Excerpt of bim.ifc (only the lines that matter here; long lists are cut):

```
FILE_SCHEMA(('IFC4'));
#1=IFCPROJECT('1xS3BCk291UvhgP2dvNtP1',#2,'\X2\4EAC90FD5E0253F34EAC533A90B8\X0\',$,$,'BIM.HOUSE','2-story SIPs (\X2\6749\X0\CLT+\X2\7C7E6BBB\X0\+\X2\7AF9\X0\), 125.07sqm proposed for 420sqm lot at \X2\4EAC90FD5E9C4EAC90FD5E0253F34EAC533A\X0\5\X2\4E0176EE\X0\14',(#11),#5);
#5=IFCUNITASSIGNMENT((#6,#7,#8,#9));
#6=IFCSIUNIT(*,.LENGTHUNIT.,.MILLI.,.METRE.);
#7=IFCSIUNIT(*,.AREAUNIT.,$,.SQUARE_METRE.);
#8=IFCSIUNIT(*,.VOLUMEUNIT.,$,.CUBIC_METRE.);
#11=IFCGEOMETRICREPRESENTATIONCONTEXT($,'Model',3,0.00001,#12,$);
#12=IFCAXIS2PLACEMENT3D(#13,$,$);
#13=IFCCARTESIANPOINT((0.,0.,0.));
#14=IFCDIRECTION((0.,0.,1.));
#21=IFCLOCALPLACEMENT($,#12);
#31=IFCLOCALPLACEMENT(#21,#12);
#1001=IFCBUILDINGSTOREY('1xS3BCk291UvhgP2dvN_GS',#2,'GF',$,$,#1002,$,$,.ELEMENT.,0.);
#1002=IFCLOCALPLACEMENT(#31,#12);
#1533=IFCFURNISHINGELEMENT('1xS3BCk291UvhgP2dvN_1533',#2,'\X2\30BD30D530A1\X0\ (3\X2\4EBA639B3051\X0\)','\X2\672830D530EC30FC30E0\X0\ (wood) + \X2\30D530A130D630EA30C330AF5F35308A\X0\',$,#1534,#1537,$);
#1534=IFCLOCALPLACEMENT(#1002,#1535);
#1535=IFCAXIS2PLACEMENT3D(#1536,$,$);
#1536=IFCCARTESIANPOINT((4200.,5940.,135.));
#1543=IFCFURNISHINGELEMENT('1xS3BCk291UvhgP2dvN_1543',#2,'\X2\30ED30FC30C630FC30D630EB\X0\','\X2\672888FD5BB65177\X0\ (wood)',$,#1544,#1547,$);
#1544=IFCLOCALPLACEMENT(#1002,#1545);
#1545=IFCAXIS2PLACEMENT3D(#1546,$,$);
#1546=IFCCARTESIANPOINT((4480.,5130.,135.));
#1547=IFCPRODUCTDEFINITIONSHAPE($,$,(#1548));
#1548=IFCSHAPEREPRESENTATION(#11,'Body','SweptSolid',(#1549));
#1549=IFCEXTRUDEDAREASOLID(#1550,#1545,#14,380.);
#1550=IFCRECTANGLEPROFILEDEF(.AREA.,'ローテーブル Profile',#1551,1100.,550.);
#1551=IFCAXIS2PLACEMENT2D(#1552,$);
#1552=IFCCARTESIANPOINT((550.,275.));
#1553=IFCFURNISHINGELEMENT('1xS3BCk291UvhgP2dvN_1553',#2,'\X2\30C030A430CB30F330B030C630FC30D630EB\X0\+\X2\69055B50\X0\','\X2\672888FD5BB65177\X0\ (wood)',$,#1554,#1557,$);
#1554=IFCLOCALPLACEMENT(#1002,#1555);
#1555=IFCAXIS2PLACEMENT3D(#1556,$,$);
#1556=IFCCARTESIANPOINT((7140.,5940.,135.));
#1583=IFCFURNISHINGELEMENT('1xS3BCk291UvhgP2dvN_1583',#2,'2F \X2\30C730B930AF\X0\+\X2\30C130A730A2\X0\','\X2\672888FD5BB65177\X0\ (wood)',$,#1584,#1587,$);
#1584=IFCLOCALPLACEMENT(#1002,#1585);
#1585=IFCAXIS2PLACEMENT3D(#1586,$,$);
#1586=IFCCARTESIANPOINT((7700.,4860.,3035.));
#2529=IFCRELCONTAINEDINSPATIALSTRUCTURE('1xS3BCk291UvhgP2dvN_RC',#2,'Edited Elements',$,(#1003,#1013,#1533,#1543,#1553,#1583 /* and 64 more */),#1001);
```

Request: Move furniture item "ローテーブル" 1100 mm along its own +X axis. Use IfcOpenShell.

```python
import ifcopenshell
import ifcopenshell.api.geometry
import ifcopenshell.util.placement
import ifcopenshell.util.unit

model = ifcopenshell.open("bim.ifc")
unit_scale = ifcopenshell.util.unit.calculate_unit_scale(model)

item = model.by_guid("1xS3BCk291UvhgP2dvN_1543")
matrix = ifcopenshell.util.placement.get_local_placement(item.ObjectPlacement)
matrix[:3, 3] += matrix[:3, 0] * 1.1 / unit_scale
ifcopenshell.api.geometry.edit_object_placement(model, product=item, matrix=matrix, is_si=False)

print(ifcopenshell.util.placement.get_local_placement(item.ObjectPlacement).round(3) + 0.0)

model.write("bim_v2.ifc")
```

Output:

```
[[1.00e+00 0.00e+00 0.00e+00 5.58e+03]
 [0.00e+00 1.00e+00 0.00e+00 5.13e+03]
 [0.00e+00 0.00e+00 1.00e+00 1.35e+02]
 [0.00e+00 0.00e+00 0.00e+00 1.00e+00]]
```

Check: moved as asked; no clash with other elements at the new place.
